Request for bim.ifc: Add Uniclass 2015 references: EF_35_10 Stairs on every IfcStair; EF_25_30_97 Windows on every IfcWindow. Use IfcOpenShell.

First a look at what the model holds.

```python
import ifcopenshell

model = ifcopenshell.open("bim.ifc")
print(model.schema)
print("classifications:", [c.Name for c in model.by_type("IfcClassification")])
for ifc_class in ("IfcDoor", "IfcRoof", "IfcStair", "IfcWall", "IfcWindow"):
    print(ifc_class, len(model.by_type(ifc_class)))
```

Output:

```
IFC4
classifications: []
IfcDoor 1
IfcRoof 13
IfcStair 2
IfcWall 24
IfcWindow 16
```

```python
import ifcopenshell
import ifcopenshell.api.classification

model = ifcopenshell.open("bim.ifc")

system = ifcopenshell.api.classification.add_classification(model, classification="Uniclass 2015")

codes = {
    "IfcStair": ("EF_35_10", "Stairs"),
    "IfcWindow": ("EF_25_30_97", "Windows"),
}
for ifc_class, (code, name) in codes.items():
    products = model.by_type(ifc_class)
    ifcopenshell.api.classification.add_reference(
        model, products=products, classification=system, identification=code, name=name
    )
    print(code, len(products))

model.write("bim_rev.ifc")
```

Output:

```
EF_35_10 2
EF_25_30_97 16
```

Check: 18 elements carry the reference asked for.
